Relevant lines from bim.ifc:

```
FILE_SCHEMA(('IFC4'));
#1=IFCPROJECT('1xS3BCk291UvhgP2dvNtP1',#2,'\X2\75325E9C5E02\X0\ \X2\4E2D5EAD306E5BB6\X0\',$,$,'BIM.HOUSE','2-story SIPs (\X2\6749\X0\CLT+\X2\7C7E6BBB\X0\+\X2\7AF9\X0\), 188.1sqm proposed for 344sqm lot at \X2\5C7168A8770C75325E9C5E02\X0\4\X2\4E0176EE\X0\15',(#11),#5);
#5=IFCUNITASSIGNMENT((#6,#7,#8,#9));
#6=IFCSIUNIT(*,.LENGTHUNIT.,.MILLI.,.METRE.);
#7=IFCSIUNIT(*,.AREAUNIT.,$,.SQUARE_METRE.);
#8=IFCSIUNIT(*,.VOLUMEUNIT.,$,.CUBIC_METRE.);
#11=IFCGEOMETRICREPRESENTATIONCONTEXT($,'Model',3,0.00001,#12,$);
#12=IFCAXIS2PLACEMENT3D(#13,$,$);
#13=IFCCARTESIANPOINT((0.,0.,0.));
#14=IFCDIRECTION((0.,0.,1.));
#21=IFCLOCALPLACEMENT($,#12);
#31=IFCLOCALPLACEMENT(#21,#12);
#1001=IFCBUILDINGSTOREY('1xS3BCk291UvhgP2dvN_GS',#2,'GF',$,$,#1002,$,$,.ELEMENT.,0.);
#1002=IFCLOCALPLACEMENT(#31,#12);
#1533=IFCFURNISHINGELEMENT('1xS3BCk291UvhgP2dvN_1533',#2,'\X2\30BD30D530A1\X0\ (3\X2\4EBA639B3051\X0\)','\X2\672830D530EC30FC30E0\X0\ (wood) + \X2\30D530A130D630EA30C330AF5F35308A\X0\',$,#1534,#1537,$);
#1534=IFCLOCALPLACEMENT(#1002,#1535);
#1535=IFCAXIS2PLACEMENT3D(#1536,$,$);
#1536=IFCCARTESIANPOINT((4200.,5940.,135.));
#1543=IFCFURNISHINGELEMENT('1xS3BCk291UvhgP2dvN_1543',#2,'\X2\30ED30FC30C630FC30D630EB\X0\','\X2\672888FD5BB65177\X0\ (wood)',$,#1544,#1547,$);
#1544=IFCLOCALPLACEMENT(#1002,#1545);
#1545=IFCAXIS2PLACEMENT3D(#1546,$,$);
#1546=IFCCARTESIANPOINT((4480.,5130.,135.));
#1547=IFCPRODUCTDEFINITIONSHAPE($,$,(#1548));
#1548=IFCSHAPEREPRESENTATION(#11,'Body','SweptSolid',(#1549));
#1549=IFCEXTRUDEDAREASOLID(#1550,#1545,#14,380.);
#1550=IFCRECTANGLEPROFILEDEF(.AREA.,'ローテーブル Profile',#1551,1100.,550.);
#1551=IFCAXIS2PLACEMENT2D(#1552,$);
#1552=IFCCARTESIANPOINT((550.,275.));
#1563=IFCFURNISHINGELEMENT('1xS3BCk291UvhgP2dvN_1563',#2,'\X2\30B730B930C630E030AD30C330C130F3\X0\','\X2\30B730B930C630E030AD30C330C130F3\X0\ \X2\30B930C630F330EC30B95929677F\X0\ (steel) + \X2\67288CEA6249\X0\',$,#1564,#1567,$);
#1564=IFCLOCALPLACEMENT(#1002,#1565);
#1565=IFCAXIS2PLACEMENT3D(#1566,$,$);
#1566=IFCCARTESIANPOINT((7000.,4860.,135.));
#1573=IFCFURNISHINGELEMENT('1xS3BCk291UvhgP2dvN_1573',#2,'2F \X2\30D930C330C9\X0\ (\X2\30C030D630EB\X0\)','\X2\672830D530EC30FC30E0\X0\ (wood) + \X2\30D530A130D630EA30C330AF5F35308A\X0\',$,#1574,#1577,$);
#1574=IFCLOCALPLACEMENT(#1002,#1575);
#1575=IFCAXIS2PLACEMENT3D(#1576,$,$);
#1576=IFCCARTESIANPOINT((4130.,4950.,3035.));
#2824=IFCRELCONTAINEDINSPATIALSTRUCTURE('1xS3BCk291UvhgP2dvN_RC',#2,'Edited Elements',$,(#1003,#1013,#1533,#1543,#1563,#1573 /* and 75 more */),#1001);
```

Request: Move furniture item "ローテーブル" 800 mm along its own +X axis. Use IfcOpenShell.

```python
import ifcopenshell
import ifcopenshell.api.geometry
import ifcopenshell.util.placement
import ifcopenshell.util.unit

model = ifcopenshell.open("bim.ifc")
unit_scale = ifcopenshell.util.unit.calculate_unit_scale(model)

item = model.by_guid("1xS3BCk291UvhgP2dvN_1543")
matrix = ifcopenshell.util.placement.get_local_placement(item.ObjectPlacement)
matrix[:3, 3] += matrix[:3, 0] * 0.8 / unit_scale
ifcopenshell.api.geometry.edit_object_placement(model, product=item, matrix=matrix, is_si=False)

print(ifcopenshell.util.placement.get_local_placement(item.ObjectPlacement).round(3) + 0.0)

model.write("bim_edited.ifc")
```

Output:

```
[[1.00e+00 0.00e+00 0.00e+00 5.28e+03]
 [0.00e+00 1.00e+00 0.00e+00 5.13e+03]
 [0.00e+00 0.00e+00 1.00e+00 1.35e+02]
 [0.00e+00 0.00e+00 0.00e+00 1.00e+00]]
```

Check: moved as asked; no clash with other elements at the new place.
